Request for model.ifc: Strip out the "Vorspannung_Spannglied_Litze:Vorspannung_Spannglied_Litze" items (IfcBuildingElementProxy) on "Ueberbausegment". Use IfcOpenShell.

First a look at what the model holds.

```python
import ifcopenshell
import ifcopenshell.util.element

model = ifcopenshell.open("model.ifc")
print(model.schema)
storey = next(s for s in model.by_type("IfcBuildingStorey") if s.Name == "Ueberbausegment")
proxies = [e for e in ifcopenshell.util.element.get_decomposition(storey) if e.is_a("IfcBuildingElementProxy")]
seen = {}
for e in proxies:
    element_type = ifcopenshell.util.element.get_type(e)
    name = element_type.Name if element_type not in (None, e) else None
    seen[name] = seen.get(name, 0) + 1
for name, count in sorted(seen.items(), key=str):
    print(count, "x", name)
```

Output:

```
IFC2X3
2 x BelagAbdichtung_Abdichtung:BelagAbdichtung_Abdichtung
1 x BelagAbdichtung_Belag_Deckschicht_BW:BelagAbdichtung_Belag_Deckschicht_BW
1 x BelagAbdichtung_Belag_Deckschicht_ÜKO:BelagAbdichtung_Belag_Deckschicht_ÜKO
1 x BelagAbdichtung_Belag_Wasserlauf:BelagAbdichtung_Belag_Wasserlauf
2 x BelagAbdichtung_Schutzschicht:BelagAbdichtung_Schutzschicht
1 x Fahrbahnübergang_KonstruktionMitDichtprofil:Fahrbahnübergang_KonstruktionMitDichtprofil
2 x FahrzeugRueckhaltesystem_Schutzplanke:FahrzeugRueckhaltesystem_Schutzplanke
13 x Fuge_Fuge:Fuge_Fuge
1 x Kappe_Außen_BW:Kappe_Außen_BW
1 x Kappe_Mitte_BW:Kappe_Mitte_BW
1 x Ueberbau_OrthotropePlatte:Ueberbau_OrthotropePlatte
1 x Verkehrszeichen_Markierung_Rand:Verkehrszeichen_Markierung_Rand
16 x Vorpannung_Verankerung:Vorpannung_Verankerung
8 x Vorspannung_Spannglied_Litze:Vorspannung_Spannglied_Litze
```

```python
import ifcopenshell
import ifcopenshell.api.root
import ifcopenshell.util.element

model = ifcopenshell.open("model.ifc")

storey = next(s for s in model.by_type("IfcBuildingStorey") if s.Name == "Ueberbausegment")
proxies = [e for e in ifcopenshell.util.element.get_decomposition(storey) if e.is_a("IfcBuildingElementProxy")]
targets = [e for e in proxies if (t := ifcopenshell.util.element.get_type(e)) not in (None, e) and t.Name == "Vorspannung_Spannglied_Litze:Vorspannung_Spannglied_Litze"]

for e in targets:
    ifcopenshell.api.root.remove_product(model, product=e)
print(len(targets), "removed")

model.write("model_edited.ifc")
```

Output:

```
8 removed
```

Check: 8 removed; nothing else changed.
